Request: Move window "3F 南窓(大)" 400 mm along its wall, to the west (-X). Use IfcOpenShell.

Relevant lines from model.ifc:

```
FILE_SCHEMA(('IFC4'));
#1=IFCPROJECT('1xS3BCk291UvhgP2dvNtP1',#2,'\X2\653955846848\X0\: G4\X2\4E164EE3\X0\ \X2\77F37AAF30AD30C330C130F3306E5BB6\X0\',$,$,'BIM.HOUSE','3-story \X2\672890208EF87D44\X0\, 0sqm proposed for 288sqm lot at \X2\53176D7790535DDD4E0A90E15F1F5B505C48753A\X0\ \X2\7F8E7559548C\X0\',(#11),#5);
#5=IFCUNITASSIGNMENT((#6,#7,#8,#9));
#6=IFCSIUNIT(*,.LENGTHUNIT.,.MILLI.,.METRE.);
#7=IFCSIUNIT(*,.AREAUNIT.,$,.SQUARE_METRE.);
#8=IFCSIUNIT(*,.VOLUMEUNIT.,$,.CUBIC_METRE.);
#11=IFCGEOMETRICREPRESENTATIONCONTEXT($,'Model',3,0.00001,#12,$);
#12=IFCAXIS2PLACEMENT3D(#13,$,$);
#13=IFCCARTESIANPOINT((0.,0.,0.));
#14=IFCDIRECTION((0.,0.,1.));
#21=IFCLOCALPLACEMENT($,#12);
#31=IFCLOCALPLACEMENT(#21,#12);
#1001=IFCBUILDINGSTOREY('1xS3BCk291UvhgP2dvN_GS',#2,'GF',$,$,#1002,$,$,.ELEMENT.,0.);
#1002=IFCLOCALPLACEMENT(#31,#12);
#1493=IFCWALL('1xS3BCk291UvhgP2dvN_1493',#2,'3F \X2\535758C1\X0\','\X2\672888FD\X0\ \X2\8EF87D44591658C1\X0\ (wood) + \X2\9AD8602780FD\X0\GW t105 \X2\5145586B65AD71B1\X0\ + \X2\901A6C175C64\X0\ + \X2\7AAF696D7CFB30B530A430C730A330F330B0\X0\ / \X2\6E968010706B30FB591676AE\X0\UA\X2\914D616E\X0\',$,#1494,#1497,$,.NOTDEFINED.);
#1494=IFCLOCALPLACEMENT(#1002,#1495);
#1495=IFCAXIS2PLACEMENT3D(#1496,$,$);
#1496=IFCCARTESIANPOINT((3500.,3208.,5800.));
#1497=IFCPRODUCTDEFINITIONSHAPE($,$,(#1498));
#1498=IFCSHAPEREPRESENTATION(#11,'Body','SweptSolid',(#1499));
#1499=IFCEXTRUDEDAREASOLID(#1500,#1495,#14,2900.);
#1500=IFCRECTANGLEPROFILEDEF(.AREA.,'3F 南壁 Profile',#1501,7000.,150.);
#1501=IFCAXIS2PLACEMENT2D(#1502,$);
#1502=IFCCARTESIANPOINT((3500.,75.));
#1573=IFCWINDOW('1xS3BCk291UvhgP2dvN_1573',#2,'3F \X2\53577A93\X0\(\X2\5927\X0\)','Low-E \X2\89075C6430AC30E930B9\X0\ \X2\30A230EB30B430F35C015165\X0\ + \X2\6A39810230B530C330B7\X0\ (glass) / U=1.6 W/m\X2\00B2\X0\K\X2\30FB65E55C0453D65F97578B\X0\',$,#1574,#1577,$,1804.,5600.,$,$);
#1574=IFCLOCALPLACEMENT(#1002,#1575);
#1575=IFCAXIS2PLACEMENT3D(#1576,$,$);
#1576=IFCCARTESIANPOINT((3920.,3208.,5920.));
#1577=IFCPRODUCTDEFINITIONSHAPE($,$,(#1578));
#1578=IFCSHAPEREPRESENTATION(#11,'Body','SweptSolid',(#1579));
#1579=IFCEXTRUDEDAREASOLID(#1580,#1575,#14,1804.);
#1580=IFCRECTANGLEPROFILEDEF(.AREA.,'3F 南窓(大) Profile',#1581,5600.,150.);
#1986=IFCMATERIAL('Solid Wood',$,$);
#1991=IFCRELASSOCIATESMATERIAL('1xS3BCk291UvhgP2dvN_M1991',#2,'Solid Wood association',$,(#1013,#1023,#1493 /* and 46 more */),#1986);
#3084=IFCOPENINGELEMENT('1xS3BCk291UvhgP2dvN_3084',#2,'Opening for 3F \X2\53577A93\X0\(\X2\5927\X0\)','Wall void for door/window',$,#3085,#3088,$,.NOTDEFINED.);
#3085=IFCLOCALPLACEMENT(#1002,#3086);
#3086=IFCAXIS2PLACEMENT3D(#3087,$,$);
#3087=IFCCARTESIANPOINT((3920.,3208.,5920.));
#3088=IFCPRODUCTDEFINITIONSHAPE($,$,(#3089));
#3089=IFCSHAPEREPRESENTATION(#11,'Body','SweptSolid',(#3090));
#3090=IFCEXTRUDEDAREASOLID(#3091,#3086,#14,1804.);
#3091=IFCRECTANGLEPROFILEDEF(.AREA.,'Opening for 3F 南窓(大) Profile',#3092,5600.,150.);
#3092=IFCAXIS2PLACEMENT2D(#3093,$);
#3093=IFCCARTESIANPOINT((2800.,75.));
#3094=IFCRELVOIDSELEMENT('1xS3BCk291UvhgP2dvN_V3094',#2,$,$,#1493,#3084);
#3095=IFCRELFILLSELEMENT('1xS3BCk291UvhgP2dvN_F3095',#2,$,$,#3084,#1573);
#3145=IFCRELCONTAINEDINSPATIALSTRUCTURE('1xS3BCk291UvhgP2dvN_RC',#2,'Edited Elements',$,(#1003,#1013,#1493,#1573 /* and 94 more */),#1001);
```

```python
import ifcopenshell
import ifcopenshell.api.geometry
import ifcopenshell.util.placement

model = ifcopenshell.open("model.ifc")

window = model.by_id(1573)
opening = window.FillsVoids[0].RelatingOpeningElement
wall = opening.VoidsElements[0].RelatingBuildingElement

wall_matrix = ifcopenshell.util.placement.get_local_placement(wall.ObjectPlacement)
shift = wall_matrix[:3, 0] * -400.0
before = ifcopenshell.util.placement.get_local_placement(window.ObjectPlacement)[:3, 3].copy()

# The window is not placed relative to its opening, so move both.
for product in (opening, window):
    matrix = ifcopenshell.util.placement.get_local_placement(product.ObjectPlacement)
    matrix[:3, 3] += shift
    ifcopenshell.api.geometry.edit_object_placement(model, product=product, matrix=matrix, is_si=False)

after = ifcopenshell.util.placement.get_local_placement(window.ObjectPlacement)[:3, 3]
print("window moved by", (after - before).round(3) + 0.0)

model.write("model_edited.ifc")
```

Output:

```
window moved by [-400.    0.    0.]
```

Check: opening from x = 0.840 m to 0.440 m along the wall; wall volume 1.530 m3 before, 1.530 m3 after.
